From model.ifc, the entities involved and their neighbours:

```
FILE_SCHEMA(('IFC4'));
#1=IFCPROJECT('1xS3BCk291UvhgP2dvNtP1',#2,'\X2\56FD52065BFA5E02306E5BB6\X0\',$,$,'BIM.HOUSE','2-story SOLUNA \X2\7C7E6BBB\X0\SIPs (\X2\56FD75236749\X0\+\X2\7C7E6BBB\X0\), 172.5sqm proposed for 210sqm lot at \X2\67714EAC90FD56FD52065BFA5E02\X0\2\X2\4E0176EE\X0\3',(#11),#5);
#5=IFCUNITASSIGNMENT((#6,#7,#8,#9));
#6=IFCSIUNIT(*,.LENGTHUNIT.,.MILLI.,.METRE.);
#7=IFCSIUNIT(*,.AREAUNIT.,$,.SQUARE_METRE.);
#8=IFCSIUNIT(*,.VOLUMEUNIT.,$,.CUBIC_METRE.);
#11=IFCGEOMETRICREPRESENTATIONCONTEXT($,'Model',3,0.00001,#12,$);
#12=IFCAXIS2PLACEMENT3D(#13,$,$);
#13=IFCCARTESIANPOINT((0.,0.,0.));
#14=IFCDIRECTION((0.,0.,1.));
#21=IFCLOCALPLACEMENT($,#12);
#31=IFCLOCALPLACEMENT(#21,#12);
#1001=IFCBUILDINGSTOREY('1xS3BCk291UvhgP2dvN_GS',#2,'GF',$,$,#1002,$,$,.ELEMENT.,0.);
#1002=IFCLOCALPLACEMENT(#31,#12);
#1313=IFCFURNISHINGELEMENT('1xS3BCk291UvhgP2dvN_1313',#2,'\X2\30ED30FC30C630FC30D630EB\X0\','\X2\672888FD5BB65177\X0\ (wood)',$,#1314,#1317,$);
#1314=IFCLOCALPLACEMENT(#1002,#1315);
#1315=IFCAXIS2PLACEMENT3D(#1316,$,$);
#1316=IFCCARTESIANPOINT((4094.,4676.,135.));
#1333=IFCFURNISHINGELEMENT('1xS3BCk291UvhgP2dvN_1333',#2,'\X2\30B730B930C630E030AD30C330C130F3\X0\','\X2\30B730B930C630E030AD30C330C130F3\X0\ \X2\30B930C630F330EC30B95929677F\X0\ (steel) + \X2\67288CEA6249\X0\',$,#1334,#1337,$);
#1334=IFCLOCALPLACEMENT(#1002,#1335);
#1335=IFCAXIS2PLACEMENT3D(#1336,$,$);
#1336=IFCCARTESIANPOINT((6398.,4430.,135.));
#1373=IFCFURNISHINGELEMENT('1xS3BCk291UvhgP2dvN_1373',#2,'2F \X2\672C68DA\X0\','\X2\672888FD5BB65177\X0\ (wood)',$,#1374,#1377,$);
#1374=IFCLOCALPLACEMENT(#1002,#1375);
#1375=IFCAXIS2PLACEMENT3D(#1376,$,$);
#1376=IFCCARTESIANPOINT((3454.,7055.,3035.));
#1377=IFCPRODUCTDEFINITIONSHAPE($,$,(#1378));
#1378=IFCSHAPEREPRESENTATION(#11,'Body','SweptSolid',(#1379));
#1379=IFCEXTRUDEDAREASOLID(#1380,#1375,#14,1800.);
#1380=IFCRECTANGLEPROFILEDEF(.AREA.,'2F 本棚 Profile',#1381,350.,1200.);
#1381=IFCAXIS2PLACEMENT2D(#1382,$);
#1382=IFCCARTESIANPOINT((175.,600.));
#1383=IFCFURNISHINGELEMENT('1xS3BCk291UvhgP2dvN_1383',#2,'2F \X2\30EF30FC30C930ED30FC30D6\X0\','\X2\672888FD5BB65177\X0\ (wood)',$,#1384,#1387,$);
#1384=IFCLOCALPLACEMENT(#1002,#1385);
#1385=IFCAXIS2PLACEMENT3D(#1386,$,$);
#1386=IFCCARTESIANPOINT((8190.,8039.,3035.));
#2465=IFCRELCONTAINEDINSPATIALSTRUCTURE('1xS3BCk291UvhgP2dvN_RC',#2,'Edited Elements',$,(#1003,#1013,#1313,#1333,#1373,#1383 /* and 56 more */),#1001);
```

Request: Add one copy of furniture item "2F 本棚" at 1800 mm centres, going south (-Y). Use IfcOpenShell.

```python
import numpy as np
import ifcopenshell
import ifcopenshell.api.geometry
import ifcopenshell.api.root
import ifcopenshell.util.element
import ifcopenshell.util.placement
import ifcopenshell.util.unit

model = ifcopenshell.open("model.ifc")
unit_scale = ifcopenshell.util.unit.calculate_unit_scale(model)


def reuse_history(source, copy):
    """copy_class also copies each property set's owner history, people and application; keep the originals."""
    for rel in copy.IsDefinedBy:
        if rel.is_a("IfcRelDefinesByProperties") and (history := rel.RelatingPropertyDefinition.OwnerHistory):
            rel.RelatingPropertyDefinition.OwnerHistory = source.OwnerHistory
            ifcopenshell.util.element.remove_deep2(model, history)


source = model.by_id(1373)
base = ifcopenshell.util.placement.get_local_placement(source.ObjectPlacement)
step = np.array([0.0, -1.0, 0.0]) * 1.8 / unit_scale

for i in range(1, 2):
    copy = ifcopenshell.api.root.copy_class(model, product=source)
    copy.Representation = ifcopenshell.util.element.copy_deep(
        model, source.Representation, exclude=["IfcGeometricRepresentationContext", "IfcRepresentationMap"]
    )
    reuse_history(source, copy)
    matrix = base.copy()
    matrix[:3, 3] += i * step
    print("added at", matrix[:3, 3].round(3) + 0.0)
    ifcopenshell.api.geometry.edit_object_placement(model, product=copy, matrix=matrix, is_si=False)

model.write("model_rev.ifc")
```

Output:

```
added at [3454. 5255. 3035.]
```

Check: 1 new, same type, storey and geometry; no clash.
